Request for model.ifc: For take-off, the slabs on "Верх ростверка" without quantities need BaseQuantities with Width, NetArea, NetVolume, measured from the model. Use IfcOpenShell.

First a look at what the model holds.

```python
import ifcopenshell
import ifcopenshell.util.element
import ifcopenshell.util.unit

model = ifcopenshell.open("model.ifc")
print(model.schema)
for unit_type in ("LENGTHUNIT", "AREAUNIT", "VOLUMEUNIT"):
    print(unit_type, ifcopenshell.util.unit.calculate_unit_scale(model, unit_type))
storey = next(s for s in model.by_type("IfcBuildingStorey") if s.Name == "Верх ростверка")
slabs = [e for e in ifcopenshell.util.element.get_decomposition(storey) if e.is_a("IfcSlab")]
for e in sorted(slabs, key=lambda e: e.id()):
    print(e.id(), e.is_a(), e.Name, list(ifcopenshell.util.element.get_psets(e, qtos_only=True)), sep=" | ")
```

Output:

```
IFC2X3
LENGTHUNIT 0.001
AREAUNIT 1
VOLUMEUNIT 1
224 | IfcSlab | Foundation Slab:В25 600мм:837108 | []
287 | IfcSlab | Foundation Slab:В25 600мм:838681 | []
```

```python
import ifcopenshell
import ifcopenshell.api.pset
import ifcopenshell.geom
import ifcopenshell.util.element
import ifcopenshell.util.shape
import ifcopenshell.util.unit

model = ifcopenshell.open("model.ifc")
unit_scale = ifcopenshell.util.unit.calculate_unit_scale(model)
area_scale = ifcopenshell.util.unit.calculate_unit_scale(model, "AREAUNIT")
volume_scale = ifcopenshell.util.unit.calculate_unit_scale(model, "VOLUMEUNIT")
settings = ifcopenshell.geom.settings()

storey = next(s for s in model.by_type("IfcBuildingStorey") if s.Name == "Верх ростверка")
slabs = [e for e in ifcopenshell.util.element.get_decomposition(storey) if e.is_a("IfcSlab")]

for e in sorted(slabs, key=lambda e: e.id()):
    if ifcopenshell.util.element.get_psets(e, qtos_only=True, should_inherit=False):
        continue
    # Geometry comes back in metres, in the element's own axes.
    shape = ifcopenshell.geom.create_shape(settings, e)
    values = {
        "Width": ifcopenshell.util.shape.get_z(shape.geometry) / unit_scale,
        "NetArea": ifcopenshell.util.shape.get_footprint_area(shape.geometry) / area_scale,
        "NetVolume": ifcopenshell.util.shape.get_volume(shape.geometry) / volume_scale,
    }
    qto = ifcopenshell.api.pset.add_qto(model, product=e, name="BaseQuantities")
    ifcopenshell.api.pset.edit_qto(model, qto=qto, properties=values)
    print(e.id(), {k: round(v, 3) for k, v in values.items()})

model.write("model_rev.ifc")
```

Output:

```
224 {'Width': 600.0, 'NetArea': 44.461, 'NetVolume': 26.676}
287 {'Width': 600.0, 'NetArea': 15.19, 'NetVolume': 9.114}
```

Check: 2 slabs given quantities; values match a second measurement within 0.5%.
